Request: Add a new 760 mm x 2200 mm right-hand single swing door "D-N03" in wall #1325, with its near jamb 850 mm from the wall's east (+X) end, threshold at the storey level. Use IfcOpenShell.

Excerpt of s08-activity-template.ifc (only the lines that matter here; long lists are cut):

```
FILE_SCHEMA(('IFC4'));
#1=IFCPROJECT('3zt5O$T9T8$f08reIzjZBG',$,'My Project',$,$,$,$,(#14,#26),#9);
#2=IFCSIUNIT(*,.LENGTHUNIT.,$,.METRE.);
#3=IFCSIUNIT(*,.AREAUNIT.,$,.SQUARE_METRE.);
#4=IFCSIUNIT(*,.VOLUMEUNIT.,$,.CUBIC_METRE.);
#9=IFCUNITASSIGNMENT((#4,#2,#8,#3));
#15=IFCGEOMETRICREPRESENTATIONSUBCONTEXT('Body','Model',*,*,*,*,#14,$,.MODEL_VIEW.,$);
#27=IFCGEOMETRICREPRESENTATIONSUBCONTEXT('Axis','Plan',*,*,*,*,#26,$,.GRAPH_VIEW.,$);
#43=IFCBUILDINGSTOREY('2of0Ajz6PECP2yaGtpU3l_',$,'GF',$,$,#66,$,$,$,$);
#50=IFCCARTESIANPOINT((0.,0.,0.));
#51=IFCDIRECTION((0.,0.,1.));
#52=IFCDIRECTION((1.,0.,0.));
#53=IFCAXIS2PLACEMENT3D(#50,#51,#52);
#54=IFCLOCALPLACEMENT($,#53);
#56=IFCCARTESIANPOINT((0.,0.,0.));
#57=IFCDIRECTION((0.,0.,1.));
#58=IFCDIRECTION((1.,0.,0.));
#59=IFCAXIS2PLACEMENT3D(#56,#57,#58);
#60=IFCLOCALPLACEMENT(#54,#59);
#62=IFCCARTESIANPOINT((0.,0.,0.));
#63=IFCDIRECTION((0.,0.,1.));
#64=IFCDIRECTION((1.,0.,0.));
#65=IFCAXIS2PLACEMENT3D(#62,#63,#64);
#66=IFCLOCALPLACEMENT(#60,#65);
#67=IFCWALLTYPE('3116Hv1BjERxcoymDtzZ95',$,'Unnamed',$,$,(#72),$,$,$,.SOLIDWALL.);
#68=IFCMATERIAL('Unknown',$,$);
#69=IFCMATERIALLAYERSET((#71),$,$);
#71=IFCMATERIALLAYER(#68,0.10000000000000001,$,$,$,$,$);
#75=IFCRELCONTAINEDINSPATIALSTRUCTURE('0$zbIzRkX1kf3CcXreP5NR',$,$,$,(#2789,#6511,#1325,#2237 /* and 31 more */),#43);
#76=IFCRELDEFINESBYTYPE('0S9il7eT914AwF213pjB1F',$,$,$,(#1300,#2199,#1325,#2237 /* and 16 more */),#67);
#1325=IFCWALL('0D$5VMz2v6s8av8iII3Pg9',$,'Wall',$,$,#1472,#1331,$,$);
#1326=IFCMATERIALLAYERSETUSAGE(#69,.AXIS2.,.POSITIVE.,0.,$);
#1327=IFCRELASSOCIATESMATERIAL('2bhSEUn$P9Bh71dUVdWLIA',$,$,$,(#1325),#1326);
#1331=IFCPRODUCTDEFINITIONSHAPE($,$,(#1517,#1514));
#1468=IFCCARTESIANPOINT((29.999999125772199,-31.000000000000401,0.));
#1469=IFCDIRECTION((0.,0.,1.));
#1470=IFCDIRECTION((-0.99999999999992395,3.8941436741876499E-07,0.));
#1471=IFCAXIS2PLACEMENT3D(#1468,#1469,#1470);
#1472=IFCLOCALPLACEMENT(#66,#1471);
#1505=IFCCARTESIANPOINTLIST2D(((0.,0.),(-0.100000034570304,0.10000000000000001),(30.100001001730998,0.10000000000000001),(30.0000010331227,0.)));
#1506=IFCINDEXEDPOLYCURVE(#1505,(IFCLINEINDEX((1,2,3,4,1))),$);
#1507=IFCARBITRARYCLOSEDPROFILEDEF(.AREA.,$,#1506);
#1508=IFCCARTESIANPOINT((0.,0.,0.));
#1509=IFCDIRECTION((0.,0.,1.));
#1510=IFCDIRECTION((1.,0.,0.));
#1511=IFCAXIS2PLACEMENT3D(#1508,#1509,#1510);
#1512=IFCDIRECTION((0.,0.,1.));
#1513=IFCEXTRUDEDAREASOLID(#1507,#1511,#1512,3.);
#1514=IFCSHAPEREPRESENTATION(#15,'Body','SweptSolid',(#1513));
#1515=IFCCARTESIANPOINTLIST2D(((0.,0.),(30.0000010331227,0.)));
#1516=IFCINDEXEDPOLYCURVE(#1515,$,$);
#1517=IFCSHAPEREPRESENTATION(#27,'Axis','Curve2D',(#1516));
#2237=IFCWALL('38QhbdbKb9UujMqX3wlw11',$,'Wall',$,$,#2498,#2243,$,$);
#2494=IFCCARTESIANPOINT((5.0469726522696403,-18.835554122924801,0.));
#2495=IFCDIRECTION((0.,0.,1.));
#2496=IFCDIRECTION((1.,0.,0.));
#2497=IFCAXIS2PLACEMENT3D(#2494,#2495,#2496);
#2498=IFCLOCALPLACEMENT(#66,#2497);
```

```python
import numpy as np
import ifcopenshell
import ifcopenshell.api.feature
import ifcopenshell.api.geometry
import ifcopenshell.api.root
import ifcopenshell.api.spatial
import ifcopenshell.geom
import ifcopenshell.util.element
import ifcopenshell.util.placement
import ifcopenshell.util.representation
import ifcopenshell.util.shape
import ifcopenshell.util.unit

model = ifcopenshell.open("s08-activity-template.ifc")
unit_scale = ifcopenshell.util.unit.calculate_unit_scale(model)
settings = ifcopenshell.geom.settings()


def volume(element):
    """Net volume in cubic metres, openings subtracted."""
    shape = ifcopenshell.geom.create_shape(settings, element)
    return ifcopenshell.util.shape.get_volume(shape.geometry)


wall = model.by_guid("0D$5VMz2v6s8av8iII3Pg9")
storey = ifcopenshell.util.element.get_container(wall, ifc_class="IfcBuildingStorey")
context = ifcopenshell.util.representation.get_context(model, "Model", "Body", "MODEL_VIEW")
before = volume(wall)

width, height, from_end, sill = 0.76, 2.2, 0.85, 0.0  # metres

# The wall runs along its own X axis, and the end named is its -X end.
wall_shape = ifcopenshell.geom.create_shape(settings, wall)
x, y, z = ifcopenshell.util.shape.get_vertices(wall_shape.geometry).T
start = x.min() + from_end
face, thickness = float(y.min()), float(y.max() - y.min())
wall_matrix = ifcopenshell.util.placement.get_local_placement(wall.ObjectPlacement)
level = ifcopenshell.util.placement.get_local_placement(storey.ObjectPlacement)[2, 3]


def in_wall(x, y):
    """Placement at x, y metres in the wall's axes, at sill height."""
    matrix = wall_matrix.copy()
    matrix[:, 3] = wall_matrix @ np.array([x / unit_scale, y / unit_scale, 0.0, 1.0])
    matrix[2, 3] = level + sill / unit_scale
    return matrix


# Opening: a box that overshoots both wall faces by 50 mm.
opening = ifcopenshell.api.root.create_entity(model, ifc_class="IfcOpeningElement", predefined_type="OPENING")
box = ifcopenshell.api.geometry.add_wall_representation(
    model, context=context, length=width, height=height, thickness=thickness + 0.1
)
ifcopenshell.api.geometry.assign_representation(model, product=opening, representation=box)
ifcopenshell.api.geometry.edit_object_placement(model, product=opening, matrix=in_wall(start, face - 0.05), is_si=False)
ifcopenshell.api.feature.add_feature(model, feature=opening, element=wall)

door = ifcopenshell.api.root.create_entity(model, ifc_class="IfcDoor", name="D-N03", predefined_type="DOOR")
door.OverallWidth, door.OverallHeight = width / unit_scale, height / unit_scale
door.OperationType = "SINGLE_SWING_RIGHT"
body = ifcopenshell.api.geometry.add_door_representation(
    model,
    context=context,
    overall_width=door.OverallWidth,
    overall_height=door.OverallHeight,
    operation_type="SINGLE_SWING_RIGHT",
    lining_properties={"LiningDepth": thickness / unit_scale, "ThresholdDepth": thickness / unit_scale},
)
ifcopenshell.api.geometry.assign_representation(model, product=door, representation=body)
ifcopenshell.api.spatial.assign_container(model, products=[door], relating_structure=storey)
ifcopenshell.api.feature.add_filling(model, opening=opening, element=door)

# The lining spans the wall, so the door starts at the wall face.
ifcopenshell.api.geometry.edit_object_placement(model, product=door, matrix=in_wall(start, face), is_si=False)

after = volume(wall)

print(f"wall volume {before:.3f} -> {after:.3f} m3")

model.write("s08-activity-template_v2.ifc")
```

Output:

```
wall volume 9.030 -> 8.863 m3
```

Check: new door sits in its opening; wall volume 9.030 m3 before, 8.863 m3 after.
